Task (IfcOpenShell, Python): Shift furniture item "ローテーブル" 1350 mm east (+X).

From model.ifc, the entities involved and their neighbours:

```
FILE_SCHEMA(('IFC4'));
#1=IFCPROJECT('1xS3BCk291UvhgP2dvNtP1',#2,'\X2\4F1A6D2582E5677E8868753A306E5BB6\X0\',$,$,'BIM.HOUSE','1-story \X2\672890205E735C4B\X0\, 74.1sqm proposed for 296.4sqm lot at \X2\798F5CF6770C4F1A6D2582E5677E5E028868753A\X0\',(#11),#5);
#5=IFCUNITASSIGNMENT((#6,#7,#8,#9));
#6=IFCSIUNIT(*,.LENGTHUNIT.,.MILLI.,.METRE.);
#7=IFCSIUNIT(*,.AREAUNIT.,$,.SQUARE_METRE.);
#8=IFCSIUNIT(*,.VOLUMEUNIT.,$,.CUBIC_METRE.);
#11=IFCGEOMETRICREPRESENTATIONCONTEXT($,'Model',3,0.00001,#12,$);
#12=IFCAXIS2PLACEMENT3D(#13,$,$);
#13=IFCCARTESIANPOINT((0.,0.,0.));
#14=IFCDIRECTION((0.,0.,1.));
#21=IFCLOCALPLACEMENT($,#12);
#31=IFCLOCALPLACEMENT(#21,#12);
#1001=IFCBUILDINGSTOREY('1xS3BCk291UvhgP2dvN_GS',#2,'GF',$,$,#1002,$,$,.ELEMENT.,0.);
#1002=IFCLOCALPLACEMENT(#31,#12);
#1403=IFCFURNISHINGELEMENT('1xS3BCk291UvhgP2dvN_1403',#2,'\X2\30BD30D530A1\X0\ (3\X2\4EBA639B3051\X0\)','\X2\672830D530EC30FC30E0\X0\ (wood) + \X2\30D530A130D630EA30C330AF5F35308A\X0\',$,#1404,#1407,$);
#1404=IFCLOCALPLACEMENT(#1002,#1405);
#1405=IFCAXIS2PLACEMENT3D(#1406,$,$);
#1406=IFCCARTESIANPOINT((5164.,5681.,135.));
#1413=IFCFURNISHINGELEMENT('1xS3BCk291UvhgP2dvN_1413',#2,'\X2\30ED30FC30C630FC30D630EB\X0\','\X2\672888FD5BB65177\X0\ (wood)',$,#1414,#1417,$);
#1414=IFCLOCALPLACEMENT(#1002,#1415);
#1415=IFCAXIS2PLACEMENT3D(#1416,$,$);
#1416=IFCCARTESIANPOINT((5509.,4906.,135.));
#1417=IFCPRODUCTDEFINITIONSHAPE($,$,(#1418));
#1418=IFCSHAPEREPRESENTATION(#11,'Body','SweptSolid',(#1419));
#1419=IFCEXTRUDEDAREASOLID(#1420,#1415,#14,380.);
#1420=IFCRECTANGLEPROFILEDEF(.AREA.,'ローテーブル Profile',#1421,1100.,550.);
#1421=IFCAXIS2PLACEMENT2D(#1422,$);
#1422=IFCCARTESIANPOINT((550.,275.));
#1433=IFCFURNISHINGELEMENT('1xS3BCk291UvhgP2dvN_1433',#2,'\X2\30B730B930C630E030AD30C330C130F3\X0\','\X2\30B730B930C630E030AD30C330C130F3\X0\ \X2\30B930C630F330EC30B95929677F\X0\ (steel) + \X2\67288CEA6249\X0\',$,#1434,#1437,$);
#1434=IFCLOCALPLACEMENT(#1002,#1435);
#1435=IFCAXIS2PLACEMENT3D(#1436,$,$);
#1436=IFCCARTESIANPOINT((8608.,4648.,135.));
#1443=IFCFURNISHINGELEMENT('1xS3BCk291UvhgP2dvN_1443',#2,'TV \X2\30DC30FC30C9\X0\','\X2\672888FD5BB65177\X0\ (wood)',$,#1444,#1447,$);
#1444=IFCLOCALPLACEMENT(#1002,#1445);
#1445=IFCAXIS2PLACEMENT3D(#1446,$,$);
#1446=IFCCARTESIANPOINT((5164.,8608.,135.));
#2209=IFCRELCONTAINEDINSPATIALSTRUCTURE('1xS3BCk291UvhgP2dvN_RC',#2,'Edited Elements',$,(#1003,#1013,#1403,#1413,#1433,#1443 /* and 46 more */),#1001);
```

```python
import ifcopenshell
import ifcopenshell.api.geometry
import ifcopenshell.util.placement

model = ifcopenshell.open("model.ifc")

item = model.by_id(1413)
matrix = ifcopenshell.util.placement.get_local_placement(item.ObjectPlacement)
matrix[0, 3] += 1350.0
ifcopenshell.api.geometry.edit_object_placement(model, product=item, matrix=matrix, is_si=False)

print(ifcopenshell.util.placement.get_local_placement(item.ObjectPlacement).round(3) + 0.0)

model.write("model_v2.ifc")
```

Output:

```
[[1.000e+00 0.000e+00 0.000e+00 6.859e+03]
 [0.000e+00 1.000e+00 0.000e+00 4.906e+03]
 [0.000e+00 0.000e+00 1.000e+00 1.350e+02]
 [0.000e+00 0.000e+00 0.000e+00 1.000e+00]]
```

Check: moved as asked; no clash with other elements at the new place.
